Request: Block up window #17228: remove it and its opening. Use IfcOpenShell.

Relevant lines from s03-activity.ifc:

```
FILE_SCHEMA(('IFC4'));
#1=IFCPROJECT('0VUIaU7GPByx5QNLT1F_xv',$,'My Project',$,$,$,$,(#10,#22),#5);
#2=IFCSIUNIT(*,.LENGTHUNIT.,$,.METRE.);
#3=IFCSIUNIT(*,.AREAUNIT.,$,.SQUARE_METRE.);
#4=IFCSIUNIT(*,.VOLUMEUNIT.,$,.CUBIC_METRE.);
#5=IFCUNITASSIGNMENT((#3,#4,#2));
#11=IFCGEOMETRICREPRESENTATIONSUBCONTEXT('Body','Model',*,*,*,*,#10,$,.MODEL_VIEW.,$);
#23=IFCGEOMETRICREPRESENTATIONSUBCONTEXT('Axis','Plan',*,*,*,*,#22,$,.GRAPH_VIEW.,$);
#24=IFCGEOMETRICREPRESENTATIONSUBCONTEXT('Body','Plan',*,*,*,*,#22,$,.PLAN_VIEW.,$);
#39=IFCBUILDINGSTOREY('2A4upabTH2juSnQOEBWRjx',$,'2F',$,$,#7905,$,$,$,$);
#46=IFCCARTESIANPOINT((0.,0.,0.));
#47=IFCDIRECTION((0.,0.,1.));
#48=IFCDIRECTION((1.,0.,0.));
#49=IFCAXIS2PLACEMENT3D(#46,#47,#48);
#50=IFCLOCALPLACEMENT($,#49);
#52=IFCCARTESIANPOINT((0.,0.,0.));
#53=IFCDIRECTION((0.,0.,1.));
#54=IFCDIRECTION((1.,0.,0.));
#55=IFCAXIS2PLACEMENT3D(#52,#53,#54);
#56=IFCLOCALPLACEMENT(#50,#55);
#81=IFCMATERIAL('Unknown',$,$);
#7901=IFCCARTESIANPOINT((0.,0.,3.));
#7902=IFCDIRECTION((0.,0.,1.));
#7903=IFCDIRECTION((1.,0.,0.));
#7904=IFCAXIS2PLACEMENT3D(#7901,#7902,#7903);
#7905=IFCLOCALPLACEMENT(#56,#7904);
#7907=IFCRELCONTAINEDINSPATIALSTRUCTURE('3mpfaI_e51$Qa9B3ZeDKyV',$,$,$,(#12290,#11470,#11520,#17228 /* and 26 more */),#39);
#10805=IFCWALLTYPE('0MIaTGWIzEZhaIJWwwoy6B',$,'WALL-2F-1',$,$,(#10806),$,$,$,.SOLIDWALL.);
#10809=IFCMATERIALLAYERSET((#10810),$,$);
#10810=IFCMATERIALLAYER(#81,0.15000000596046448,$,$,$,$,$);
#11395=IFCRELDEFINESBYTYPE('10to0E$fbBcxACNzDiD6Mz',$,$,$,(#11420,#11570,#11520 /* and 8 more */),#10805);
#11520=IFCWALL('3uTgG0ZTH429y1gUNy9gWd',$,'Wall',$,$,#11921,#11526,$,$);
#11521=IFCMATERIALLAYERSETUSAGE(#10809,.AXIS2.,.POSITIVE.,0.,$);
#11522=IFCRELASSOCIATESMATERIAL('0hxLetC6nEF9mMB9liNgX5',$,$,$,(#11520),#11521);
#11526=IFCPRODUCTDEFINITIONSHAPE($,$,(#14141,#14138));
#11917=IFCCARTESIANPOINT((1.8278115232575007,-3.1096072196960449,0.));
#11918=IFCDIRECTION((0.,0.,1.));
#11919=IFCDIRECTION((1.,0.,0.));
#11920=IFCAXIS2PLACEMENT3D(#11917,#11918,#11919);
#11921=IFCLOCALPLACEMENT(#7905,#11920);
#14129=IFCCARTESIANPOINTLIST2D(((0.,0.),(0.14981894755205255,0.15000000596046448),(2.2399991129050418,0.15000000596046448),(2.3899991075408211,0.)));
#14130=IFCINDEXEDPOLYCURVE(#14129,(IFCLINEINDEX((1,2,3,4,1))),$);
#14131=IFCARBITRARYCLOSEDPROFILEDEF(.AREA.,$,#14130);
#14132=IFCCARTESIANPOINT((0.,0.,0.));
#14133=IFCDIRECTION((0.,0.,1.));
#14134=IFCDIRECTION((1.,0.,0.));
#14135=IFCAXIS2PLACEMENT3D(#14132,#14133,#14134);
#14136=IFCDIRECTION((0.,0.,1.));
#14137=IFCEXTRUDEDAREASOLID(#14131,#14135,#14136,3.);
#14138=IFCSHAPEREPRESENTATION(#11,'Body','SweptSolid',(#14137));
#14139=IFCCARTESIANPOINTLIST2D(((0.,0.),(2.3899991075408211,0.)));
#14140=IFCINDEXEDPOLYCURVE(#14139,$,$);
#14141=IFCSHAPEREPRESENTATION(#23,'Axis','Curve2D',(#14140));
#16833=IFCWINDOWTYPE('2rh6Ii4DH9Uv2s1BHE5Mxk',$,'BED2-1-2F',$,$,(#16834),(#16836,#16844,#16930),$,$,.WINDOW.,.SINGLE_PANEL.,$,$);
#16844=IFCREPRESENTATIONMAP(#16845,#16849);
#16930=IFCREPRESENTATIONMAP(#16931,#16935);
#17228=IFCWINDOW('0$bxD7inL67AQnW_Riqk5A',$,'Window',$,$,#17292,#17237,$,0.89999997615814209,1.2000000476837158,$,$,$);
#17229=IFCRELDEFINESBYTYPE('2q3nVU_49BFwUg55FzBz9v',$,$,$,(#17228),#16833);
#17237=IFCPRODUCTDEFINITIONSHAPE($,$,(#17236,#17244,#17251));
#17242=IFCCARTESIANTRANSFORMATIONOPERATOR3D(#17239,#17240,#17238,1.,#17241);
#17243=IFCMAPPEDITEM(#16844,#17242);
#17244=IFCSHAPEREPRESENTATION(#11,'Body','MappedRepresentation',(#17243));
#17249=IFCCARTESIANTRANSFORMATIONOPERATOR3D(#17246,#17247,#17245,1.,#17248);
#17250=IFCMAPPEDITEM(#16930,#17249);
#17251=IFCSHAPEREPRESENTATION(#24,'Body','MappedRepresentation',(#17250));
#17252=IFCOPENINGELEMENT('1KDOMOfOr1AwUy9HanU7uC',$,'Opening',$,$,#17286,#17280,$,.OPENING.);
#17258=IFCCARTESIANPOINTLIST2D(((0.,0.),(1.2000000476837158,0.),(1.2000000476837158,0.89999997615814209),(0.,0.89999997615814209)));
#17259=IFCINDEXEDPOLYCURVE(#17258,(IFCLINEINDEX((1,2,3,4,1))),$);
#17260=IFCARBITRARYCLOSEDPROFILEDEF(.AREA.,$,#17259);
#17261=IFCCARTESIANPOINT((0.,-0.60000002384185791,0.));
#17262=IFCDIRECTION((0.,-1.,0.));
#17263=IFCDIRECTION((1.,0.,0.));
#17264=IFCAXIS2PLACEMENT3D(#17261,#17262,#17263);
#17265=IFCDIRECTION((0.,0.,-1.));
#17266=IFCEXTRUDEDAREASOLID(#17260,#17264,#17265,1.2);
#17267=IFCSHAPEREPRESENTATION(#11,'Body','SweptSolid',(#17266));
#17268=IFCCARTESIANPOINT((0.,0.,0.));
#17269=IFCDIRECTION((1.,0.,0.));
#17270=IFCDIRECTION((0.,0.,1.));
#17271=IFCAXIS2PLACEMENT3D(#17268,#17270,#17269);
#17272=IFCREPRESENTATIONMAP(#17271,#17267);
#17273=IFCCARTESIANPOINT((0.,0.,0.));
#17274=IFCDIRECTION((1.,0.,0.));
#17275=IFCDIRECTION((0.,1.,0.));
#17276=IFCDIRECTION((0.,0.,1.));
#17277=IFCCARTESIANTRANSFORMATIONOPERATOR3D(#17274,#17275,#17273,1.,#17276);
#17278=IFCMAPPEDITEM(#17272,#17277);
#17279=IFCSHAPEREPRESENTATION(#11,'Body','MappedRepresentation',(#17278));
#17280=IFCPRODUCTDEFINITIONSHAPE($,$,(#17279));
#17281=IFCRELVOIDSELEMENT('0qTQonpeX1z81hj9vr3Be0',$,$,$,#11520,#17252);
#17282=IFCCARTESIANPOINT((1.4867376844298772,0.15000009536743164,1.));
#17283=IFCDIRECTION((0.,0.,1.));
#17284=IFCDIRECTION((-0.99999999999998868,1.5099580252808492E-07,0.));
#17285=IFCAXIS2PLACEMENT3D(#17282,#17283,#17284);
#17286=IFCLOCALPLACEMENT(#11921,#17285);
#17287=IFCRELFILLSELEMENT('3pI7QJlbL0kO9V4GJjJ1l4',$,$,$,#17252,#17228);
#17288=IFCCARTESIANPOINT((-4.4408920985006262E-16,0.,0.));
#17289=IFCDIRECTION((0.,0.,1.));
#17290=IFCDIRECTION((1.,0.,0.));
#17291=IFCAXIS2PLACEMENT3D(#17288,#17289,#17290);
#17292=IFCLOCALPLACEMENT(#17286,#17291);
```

```python
import ifcopenshell
import ifcopenshell.api.feature
import ifcopenshell.api.root
import ifcopenshell.geom
import ifcopenshell.util.shape

model = ifcopenshell.open("s03-activity.ifc")
settings = ifcopenshell.geom.settings()


def volume(element):
    """Net volume in cubic metres, openings subtracted."""
    shape = ifcopenshell.geom.create_shape(settings, element)
    return ifcopenshell.util.shape.get_volume(shape.geometry)


window = model.by_guid("0$bxD7inL67AQnW_Riqk5A")
opening = window.FillsVoids[0].RelatingOpeningElement
wall = opening.VoidsElements[0].RelatingBuildingElement
before = volume(wall)

ifcopenshell.api.root.remove_product(model, product=window)
ifcopenshell.api.feature.remove_feature(model, feature=opening)

after = volume(wall)

print(f"wall volume {before:.3f} -> {after:.3f} m3")

model.write("s03-activity_rev.ifc")
```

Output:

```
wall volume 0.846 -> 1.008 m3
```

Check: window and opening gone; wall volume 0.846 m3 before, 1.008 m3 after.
